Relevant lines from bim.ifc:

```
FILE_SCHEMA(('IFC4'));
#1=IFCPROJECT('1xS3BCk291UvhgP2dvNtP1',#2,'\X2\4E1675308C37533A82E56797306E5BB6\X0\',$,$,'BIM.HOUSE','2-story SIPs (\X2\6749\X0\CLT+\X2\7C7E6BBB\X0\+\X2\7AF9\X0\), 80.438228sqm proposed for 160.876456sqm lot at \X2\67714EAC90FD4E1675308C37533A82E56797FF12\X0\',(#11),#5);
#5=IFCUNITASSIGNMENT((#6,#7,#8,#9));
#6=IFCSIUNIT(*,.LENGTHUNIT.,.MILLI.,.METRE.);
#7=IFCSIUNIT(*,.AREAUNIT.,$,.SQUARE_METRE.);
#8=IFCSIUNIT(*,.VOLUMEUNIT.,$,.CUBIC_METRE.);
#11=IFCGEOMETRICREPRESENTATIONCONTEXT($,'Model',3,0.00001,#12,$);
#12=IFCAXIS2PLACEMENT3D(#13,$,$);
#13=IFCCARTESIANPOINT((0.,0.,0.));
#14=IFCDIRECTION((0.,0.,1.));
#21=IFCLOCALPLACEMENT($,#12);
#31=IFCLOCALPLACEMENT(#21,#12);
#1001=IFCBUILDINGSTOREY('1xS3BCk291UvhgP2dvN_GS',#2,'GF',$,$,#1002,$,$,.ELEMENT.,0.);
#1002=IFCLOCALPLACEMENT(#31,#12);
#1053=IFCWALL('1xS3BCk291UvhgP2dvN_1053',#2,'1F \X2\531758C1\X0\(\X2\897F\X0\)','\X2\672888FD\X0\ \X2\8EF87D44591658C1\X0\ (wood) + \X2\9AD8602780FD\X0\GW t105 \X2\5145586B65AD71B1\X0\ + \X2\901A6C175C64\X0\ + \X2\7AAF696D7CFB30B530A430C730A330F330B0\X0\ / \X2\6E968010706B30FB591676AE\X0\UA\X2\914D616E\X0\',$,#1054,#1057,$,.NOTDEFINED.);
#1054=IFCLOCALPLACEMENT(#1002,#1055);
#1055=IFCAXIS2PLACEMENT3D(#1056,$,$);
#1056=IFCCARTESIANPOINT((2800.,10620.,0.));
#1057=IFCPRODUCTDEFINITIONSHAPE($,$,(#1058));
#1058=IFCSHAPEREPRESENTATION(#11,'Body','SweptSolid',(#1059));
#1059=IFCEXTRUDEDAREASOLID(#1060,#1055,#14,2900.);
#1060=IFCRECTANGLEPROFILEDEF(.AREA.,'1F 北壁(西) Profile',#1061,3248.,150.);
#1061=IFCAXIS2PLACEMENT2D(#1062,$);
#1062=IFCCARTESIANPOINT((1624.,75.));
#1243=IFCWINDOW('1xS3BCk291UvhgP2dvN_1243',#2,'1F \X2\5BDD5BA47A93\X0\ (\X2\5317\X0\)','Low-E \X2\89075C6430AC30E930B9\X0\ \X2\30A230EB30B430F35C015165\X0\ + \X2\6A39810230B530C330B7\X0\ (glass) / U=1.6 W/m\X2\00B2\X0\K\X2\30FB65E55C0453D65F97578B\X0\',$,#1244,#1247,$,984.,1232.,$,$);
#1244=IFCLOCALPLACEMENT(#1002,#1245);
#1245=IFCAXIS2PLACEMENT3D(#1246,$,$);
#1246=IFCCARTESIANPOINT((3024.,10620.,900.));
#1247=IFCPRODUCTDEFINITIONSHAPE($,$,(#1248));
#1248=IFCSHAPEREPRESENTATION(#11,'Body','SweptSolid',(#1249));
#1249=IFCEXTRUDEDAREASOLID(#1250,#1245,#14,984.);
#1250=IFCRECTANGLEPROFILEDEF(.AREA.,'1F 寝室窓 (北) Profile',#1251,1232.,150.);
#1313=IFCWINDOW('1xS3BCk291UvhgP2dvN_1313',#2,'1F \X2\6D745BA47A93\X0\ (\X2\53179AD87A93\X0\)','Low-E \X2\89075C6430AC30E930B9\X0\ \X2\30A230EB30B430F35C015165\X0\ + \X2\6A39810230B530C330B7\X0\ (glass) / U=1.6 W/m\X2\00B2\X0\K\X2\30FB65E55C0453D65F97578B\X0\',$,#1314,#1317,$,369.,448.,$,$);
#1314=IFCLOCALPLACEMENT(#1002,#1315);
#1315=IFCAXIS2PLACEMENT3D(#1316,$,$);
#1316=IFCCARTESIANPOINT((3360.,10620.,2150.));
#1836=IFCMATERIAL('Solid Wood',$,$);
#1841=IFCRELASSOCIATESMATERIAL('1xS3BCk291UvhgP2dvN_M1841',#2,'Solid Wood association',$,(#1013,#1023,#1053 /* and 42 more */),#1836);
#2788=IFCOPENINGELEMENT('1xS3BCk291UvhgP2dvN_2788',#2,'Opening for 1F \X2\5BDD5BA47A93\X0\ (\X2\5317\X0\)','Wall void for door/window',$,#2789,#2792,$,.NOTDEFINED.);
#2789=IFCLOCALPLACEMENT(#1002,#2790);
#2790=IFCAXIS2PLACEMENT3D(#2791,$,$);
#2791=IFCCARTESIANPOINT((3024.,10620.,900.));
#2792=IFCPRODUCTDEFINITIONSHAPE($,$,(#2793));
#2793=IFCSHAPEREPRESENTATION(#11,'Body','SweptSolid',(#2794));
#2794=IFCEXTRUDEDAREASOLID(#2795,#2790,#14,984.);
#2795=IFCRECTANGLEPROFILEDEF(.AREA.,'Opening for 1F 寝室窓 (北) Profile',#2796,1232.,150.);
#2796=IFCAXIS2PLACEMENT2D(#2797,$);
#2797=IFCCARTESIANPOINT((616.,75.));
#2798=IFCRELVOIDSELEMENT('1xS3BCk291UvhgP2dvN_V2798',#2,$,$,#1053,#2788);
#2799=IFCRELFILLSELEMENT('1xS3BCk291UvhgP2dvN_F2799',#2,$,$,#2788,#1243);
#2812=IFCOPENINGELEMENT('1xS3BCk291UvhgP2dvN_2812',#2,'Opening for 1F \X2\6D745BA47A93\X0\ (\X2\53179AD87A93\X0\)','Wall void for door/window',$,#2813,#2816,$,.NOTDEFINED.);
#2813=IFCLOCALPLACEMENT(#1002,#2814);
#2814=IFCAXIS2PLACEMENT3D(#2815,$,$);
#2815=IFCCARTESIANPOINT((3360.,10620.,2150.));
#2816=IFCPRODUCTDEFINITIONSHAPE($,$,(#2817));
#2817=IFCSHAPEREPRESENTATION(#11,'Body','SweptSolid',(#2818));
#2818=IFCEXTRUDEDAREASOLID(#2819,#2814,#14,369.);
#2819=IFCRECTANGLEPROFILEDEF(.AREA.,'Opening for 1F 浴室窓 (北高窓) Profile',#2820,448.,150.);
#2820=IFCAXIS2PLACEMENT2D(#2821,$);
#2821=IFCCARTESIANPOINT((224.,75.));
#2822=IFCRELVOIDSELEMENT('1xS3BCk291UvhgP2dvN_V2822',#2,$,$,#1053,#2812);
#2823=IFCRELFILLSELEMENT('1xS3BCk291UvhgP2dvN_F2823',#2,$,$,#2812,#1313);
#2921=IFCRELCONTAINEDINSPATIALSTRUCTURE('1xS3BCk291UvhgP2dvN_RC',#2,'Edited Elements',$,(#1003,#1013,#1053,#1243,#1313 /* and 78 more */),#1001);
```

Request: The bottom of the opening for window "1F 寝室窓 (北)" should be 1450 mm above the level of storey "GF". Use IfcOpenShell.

```python
import numpy as np
import ifcopenshell
import ifcopenshell.api.geometry
import ifcopenshell.geom
import ifcopenshell.util.element
import ifcopenshell.util.placement
import ifcopenshell.util.shape
import ifcopenshell.util.unit

model = ifcopenshell.open("bim.ifc")
unit_scale = ifcopenshell.util.unit.calculate_unit_scale(model)

window = model.by_id(1243)
opening = window.FillsVoids[0].RelatingOpeningElement
storey = ifcopenshell.util.element.get_container(window, ifc_class="IfcBuildingStorey")
level = ifcopenshell.util.placement.get_local_placement(storey.ObjectPlacement)[2, 3]

# The opening's origin need not be at the sill, so measure its lowest point.
shape = ifcopenshell.geom.create_shape(ifcopenshell.geom.settings(), opening)
bottom = ifcopenshell.util.shape.get_shape_bottom_elevation(shape, shape.geometry) / unit_scale
dz = level + 1450.0 - bottom

shift = np.array([0.0, 0.0, dz])
# The window is not placed relative to its opening, so move both.
for product in (opening, window):
    matrix = ifcopenshell.util.placement.get_local_placement(product.ObjectPlacement)
    matrix[:3, 3] += shift
    ifcopenshell.api.geometry.edit_object_placement(model, product=product, matrix=matrix, is_si=False)

print(f"moved by {dz * unit_scale:+.3f} m")

model.write("bim_edited.ifc")
```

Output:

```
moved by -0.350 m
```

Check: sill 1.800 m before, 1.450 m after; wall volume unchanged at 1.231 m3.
